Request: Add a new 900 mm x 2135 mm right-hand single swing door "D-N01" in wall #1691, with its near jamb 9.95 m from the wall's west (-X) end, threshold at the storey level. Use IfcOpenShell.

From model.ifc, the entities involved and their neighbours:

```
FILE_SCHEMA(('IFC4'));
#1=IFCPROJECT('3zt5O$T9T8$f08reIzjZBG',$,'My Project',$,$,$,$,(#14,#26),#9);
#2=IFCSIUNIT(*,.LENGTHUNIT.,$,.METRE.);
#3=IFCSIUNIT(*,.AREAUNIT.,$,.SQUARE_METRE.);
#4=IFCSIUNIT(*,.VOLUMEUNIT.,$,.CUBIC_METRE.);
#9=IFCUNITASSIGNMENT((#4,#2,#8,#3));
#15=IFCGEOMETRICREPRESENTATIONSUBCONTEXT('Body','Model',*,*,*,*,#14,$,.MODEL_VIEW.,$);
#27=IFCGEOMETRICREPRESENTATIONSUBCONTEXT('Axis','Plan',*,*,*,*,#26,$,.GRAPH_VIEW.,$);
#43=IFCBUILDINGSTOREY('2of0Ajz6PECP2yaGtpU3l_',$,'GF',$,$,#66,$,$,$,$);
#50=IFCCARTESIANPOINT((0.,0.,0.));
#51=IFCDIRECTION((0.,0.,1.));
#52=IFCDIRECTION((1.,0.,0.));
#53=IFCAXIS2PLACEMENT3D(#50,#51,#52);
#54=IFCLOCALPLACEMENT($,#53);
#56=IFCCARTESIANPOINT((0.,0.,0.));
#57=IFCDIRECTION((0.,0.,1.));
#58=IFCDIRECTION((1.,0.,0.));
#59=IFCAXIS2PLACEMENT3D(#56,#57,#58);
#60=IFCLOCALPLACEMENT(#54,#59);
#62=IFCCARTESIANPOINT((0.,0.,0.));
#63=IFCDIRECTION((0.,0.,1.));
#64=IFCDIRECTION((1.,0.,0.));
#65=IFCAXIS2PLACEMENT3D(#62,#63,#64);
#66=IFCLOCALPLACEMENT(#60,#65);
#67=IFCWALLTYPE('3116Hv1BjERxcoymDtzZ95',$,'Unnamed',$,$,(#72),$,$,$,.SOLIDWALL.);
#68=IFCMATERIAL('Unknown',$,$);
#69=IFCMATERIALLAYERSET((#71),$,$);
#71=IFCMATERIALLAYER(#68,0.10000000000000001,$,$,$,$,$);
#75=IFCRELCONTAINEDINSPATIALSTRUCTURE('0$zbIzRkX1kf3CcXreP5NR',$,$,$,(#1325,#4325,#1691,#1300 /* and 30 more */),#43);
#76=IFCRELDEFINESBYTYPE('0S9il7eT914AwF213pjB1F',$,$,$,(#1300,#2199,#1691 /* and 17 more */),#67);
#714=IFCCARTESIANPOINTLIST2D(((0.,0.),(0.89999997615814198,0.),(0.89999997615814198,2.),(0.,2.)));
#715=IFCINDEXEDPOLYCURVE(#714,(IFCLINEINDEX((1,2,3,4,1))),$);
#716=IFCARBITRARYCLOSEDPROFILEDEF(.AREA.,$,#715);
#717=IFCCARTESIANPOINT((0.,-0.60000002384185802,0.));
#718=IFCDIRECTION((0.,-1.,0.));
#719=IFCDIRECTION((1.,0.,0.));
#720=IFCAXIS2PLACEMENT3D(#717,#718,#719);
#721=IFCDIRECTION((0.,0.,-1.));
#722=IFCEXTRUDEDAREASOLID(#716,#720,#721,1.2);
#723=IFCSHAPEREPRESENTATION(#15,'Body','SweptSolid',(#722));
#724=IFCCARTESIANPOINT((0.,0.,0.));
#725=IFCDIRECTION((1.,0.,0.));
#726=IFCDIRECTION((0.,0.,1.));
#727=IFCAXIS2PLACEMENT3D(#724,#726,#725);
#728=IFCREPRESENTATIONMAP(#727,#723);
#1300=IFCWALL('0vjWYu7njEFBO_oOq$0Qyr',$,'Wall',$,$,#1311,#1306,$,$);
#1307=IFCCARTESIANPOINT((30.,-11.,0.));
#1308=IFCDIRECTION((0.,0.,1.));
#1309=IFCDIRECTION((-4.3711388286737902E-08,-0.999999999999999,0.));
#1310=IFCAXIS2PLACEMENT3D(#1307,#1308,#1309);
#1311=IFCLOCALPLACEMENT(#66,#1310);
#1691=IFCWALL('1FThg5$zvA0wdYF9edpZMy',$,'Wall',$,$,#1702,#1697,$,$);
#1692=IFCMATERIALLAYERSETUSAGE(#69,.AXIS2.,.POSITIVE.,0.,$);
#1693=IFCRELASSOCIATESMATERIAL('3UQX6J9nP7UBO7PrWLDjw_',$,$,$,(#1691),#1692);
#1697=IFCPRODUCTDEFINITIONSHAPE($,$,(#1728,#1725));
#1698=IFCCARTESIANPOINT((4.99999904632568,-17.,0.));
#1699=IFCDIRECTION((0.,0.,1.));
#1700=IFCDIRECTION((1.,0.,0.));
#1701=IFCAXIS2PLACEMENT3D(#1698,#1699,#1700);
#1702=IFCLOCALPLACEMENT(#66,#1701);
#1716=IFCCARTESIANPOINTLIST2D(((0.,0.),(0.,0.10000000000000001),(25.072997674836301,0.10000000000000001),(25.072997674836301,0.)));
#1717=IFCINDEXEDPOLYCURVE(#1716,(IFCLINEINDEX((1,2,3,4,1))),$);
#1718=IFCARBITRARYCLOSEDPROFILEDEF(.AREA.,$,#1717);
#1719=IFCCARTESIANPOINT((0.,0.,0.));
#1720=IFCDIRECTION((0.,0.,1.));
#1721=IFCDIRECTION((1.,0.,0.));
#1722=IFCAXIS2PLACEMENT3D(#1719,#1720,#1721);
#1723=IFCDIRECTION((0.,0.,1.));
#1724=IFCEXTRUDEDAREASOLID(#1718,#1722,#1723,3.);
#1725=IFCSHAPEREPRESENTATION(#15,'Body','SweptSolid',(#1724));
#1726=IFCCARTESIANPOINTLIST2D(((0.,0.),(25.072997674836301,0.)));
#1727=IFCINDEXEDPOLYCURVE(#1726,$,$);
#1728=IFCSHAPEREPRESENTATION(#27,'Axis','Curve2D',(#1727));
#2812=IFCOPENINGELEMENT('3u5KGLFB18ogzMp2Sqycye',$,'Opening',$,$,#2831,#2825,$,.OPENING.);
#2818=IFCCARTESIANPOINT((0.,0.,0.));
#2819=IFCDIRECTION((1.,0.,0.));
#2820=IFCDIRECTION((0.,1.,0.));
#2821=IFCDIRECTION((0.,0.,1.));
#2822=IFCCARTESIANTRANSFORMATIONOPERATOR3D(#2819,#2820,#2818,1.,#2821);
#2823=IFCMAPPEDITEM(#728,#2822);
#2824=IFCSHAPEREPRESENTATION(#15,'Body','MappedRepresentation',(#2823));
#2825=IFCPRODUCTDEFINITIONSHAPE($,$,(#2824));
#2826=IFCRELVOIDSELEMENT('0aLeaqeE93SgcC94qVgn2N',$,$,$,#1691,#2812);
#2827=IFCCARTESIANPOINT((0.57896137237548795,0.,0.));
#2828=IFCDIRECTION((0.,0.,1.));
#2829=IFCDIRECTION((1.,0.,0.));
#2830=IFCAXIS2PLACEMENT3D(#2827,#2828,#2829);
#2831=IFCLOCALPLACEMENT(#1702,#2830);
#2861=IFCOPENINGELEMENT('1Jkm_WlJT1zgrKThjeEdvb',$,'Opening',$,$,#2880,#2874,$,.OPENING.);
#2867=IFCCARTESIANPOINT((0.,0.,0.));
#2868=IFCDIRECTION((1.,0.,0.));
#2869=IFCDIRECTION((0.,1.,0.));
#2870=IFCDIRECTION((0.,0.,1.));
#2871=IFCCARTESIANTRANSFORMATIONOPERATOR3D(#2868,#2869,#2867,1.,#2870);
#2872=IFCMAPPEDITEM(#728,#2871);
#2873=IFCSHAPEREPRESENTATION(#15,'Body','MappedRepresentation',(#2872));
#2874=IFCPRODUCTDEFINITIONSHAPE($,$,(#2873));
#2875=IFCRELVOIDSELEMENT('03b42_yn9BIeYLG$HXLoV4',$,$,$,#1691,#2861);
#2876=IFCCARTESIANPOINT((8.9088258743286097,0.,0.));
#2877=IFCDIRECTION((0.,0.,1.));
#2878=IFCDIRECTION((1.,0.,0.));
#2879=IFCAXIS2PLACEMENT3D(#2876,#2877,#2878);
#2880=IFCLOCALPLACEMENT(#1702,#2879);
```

```python
import numpy as np
import ifcopenshell
import ifcopenshell.api.feature
import ifcopenshell.api.geometry
import ifcopenshell.api.root
import ifcopenshell.api.spatial
import ifcopenshell.geom
import ifcopenshell.util.element
import ifcopenshell.util.placement
import ifcopenshell.util.representation
import ifcopenshell.util.shape
import ifcopenshell.util.unit

model = ifcopenshell.open("model.ifc")
unit_scale = ifcopenshell.util.unit.calculate_unit_scale(model)
settings = ifcopenshell.geom.settings()


def volume(element):
    """Net volume in cubic metres, openings subtracted."""
    shape = ifcopenshell.geom.create_shape(settings, element)
    return ifcopenshell.util.shape.get_volume(shape.geometry)


wall = model.by_id(1691)
storey = ifcopenshell.util.element.get_container(wall, ifc_class="IfcBuildingStorey")
context = ifcopenshell.util.representation.get_context(model, "Model", "Body", "MODEL_VIEW")
before = volume(wall)

width, height, from_end, sill = 0.9, 2.135, 9.95, 0.0  # metres

# The wall runs along its own X axis, and the end named is its -X end.
wall_shape = ifcopenshell.geom.create_shape(settings, wall)
x, y, z = ifcopenshell.util.shape.get_vertices(wall_shape.geometry).T
start = x.min() + from_end
face, thickness = float(y.min()), float(y.max() - y.min())
wall_matrix = ifcopenshell.util.placement.get_local_placement(wall.ObjectPlacement)
level = ifcopenshell.util.placement.get_local_placement(storey.ObjectPlacement)[2, 3]


def in_wall(x, y):
    """Placement at x, y metres in the wall's axes, at sill height."""
    matrix = wall_matrix.copy()
    matrix[:, 3] = wall_matrix @ np.array([x / unit_scale, y / unit_scale, 0.0, 1.0])
    matrix[2, 3] = level + sill / unit_scale
    return matrix


# Opening: a box that overshoots both wall faces by 50 mm.
opening = ifcopenshell.api.root.create_entity(model, ifc_class="IfcOpeningElement", predefined_type="OPENING")
box = ifcopenshell.api.geometry.add_wall_representation(
    model, context=context, length=width, height=height, thickness=thickness + 0.1
)
ifcopenshell.api.geometry.assign_representation(model, product=opening, representation=box)
ifcopenshell.api.geometry.edit_object_placement(model, product=opening, matrix=in_wall(start, face - 0.05), is_si=False)
ifcopenshell.api.feature.add_feature(model, feature=opening, element=wall)

door = ifcopenshell.api.root.create_entity(model, ifc_class="IfcDoor", name="D-N01", predefined_type="DOOR")
door.OverallWidth, door.OverallHeight = width / unit_scale, height / unit_scale
door.OperationType = "SINGLE_SWING_RIGHT"
body = ifcopenshell.api.geometry.add_door_representation(
    model,
    context=context,
    overall_width=door.OverallWidth,
    overall_height=door.OverallHeight,
    operation_type="SINGLE_SWING_RIGHT",
    lining_properties={"LiningDepth": thickness / unit_scale, "ThresholdDepth": thickness / unit_scale},
)
ifcopenshell.api.geometry.assign_representation(model, product=door, representation=body)
ifcopenshell.api.spatial.assign_container(model, products=[door], relating_structure=storey)
ifcopenshell.api.feature.add_filling(model, opening=opening, element=door)

# The lining spans the wall, so the door starts at the wall face.
ifcopenshell.api.geometry.edit_object_placement(model, product=door, matrix=in_wall(start, face), is_si=False)

after = volume(wall)

print(f"wall volume {before:.3f} -> {after:.3f} m3")

model.write("model-out.ifc")
```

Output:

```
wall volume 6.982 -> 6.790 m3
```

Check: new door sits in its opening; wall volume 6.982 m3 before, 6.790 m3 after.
